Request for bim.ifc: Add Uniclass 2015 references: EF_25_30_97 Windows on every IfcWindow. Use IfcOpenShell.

First a look at what the model holds.

```python
import ifcopenshell

model = ifcopenshell.open("bim.ifc")
print(model.schema)
print("classifications:", [c.Name for c in model.by_type("IfcClassification")])
for ifc_class in ("IfcDoor", "IfcRoof", "IfcStair", "IfcWall", "IfcWindow"):
    print(ifc_class, len(model.by_type(ifc_class)))
```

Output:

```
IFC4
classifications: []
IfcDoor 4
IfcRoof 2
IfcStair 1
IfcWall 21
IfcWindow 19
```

```python
import ifcopenshell
import ifcopenshell.api.classification

model = ifcopenshell.open("bim.ifc")

system = ifcopenshell.api.classification.add_classification(model, classification="Uniclass 2015")

codes = {
    "IfcWindow": ("EF_25_30_97", "Windows"),
}
for ifc_class, (code, name) in codes.items():
    products = model.by_type(ifc_class)
    ifcopenshell.api.classification.add_reference(
        model, products=products, classification=system, identification=code, name=name
    )
    print(code, len(products))

model.write("bim-out.ifc")
```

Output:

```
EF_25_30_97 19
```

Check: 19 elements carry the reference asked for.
